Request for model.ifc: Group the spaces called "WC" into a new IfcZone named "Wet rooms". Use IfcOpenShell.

First a look at what the model holds.

```python
import ifcopenshell

model = ifcopenshell.open("model.ifc")
print(model.schema)
seen = {}
for space in model.by_type("IfcSpace"):
    seen[space.LongName] = seen.get(space.LongName, 0) + 1
for name, count in sorted(seen.items(), key=str):
    print(count, "x", name)
print("zones:", [z.Name for z in model.by_type("IfcZone")][:20])
```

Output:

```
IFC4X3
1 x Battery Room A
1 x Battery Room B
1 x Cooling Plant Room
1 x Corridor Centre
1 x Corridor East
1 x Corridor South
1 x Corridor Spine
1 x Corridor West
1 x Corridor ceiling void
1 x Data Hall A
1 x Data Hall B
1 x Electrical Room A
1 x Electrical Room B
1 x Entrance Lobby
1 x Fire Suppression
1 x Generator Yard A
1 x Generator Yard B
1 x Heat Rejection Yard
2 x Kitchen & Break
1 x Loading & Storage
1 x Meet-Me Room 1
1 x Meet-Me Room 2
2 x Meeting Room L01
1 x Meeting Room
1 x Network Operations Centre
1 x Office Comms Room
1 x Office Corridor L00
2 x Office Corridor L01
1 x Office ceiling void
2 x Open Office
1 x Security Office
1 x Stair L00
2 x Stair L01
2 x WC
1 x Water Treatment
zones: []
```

```python
import ifcopenshell
import ifcopenshell.api.group
import ifcopenshell.api.root

model = ifcopenshell.open("model.ifc")

names = {"WC"}
spaces = [s for s in model.by_type("IfcSpace") if s.LongName in names]

zone = ifcopenshell.api.root.create_entity(model, ifc_class="IfcZone", name="Wet rooms")
ifcopenshell.api.group.assign_group(model, products=spaces, group=zone)
print(len(spaces), "spaces in", zone.Name)

model.write("model-out.ifc")
```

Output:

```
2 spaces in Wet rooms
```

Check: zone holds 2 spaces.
